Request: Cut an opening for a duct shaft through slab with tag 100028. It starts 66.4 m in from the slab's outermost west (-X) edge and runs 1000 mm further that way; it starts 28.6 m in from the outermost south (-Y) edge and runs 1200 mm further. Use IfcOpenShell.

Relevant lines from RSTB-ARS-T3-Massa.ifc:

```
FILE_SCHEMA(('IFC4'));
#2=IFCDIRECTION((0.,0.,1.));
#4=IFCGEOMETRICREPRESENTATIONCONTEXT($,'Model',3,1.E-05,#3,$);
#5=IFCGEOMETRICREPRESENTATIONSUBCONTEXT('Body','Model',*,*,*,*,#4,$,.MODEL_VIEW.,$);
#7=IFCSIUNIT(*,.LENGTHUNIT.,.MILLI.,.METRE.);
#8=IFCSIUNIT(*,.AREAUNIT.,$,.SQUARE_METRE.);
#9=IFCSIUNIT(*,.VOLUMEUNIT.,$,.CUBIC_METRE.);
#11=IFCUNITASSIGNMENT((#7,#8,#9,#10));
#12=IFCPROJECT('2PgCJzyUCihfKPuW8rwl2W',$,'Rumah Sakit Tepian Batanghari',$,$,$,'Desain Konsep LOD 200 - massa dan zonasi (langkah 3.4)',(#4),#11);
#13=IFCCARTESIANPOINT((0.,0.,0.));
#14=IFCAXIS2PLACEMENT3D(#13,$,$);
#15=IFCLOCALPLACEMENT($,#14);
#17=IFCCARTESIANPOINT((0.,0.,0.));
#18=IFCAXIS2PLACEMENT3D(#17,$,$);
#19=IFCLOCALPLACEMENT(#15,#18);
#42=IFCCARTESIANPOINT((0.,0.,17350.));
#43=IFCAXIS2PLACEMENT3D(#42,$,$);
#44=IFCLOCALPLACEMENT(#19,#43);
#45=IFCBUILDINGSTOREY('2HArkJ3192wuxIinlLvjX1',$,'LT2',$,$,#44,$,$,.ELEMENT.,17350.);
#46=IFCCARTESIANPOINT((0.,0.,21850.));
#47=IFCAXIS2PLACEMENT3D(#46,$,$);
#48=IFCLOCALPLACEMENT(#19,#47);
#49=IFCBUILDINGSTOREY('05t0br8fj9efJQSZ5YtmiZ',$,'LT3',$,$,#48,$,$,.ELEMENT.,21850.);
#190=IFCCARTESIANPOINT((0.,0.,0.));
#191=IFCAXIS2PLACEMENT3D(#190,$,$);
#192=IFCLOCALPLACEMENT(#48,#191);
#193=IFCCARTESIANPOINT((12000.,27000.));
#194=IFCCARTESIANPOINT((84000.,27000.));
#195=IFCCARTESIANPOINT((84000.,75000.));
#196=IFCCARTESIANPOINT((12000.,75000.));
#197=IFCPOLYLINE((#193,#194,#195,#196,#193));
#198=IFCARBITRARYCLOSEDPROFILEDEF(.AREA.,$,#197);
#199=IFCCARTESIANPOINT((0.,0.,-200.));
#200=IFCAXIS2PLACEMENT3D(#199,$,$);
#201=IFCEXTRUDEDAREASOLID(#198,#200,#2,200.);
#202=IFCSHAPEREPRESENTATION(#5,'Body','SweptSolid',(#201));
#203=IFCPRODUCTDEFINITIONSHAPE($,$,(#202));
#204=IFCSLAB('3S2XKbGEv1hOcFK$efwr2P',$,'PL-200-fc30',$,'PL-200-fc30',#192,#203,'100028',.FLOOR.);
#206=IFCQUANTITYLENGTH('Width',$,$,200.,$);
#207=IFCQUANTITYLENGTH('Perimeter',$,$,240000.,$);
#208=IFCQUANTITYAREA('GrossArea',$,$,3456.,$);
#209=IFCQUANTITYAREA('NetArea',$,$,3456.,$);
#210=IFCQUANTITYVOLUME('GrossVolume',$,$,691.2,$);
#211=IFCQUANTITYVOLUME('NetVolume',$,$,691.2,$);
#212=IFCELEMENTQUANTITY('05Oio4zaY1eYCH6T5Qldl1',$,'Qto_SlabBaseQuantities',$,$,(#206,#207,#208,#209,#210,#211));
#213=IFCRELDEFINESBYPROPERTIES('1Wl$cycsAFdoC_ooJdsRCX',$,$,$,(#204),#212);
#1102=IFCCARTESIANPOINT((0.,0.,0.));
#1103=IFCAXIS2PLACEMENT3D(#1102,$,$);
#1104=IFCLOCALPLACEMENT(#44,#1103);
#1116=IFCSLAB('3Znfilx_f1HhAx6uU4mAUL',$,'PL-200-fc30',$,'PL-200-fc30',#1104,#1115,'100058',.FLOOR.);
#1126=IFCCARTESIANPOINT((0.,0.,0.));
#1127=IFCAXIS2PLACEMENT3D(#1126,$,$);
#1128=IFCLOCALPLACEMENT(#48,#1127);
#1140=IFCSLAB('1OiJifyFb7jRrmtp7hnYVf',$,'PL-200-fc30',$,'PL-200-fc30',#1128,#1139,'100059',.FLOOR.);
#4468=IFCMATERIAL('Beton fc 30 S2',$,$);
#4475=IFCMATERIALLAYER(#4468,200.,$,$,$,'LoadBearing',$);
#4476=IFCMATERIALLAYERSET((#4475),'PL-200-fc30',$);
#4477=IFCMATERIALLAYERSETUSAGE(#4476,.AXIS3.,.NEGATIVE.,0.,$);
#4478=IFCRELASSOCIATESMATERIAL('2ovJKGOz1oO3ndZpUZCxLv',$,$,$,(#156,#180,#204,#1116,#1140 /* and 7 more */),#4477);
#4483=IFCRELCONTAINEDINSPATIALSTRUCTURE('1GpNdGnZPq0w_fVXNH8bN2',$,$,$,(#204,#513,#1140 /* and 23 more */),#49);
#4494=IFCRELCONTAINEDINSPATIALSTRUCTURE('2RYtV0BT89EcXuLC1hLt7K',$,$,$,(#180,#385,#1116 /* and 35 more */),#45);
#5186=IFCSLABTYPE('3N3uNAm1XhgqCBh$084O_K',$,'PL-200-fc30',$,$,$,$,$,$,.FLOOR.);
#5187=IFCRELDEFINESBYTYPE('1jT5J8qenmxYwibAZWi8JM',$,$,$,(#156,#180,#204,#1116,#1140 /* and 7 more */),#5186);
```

```python
import numpy as np
import ifcopenshell
import ifcopenshell.api.feature
import ifcopenshell.api.geometry
import ifcopenshell.api.pset
import ifcopenshell.api.root
import ifcopenshell.geom
import ifcopenshell.util.element
import ifcopenshell.util.placement
import ifcopenshell.util.representation
import ifcopenshell.util.shape
import ifcopenshell.util.unit

model = ifcopenshell.open("RSTB-ARS-T3-Massa.ifc")
unit_scale = ifcopenshell.util.unit.calculate_unit_scale(model)
area_scale = ifcopenshell.util.unit.calculate_unit_scale(model, "AREAUNIT")
volume_scale = ifcopenshell.util.unit.calculate_unit_scale(model, "VOLUMEUNIT")
settings = ifcopenshell.geom.settings()


def volume(element):
    """Net volume in cubic metres, openings subtracted."""
    shape = ifcopenshell.geom.create_shape(settings, element)
    return ifcopenshell.util.shape.get_volume(shape.geometry)


slab = model.by_guid("3S2XKbGEv1hOcFK$efwr2P")
before = volume(slab)

# Extent in the slab's own axes, in metres. The edges named are its -X and -Y sides.
slab_shape = ifcopenshell.geom.create_shape(settings, slab)
vertices = ifcopenshell.util.shape.get_vertices(slab_shape.geometry)
x_min, y_min, bottom = vertices.min(axis=0)
top = vertices[:, 2].max()

opening = ifcopenshell.api.root.create_entity(model, ifc_class="IfcOpeningElement", name="Duct shaft opening", predefined_type="OPENING")
context = ifcopenshell.util.representation.get_context(model, "Model", "Body", "MODEL_VIEW")
width, depth = 1, 1.2
outline = [(0.0, 0.0), (width, 0.0), (width, depth), (0.0, depth), (0.0, 0.0)]
# Overshoot both faces by 50 mm so the cut is clean.
shape = ifcopenshell.api.geometry.add_slab_representation(
    model, context=context, depth=top - bottom + 0.1, polyline=outline
)
ifcopenshell.api.geometry.assign_representation(model, product=opening, representation=shape)

matrix = ifcopenshell.util.placement.get_local_placement(slab.ObjectPlacement)
matrix[:, 3] = matrix @ np.append(np.array([x_min + 66.4, y_min + 28.6, bottom - 0.05]) / unit_scale, 1.0)
ifcopenshell.api.geometry.edit_object_placement(model, product=opening, matrix=matrix, is_si=False)
ifcopenshell.api.feature.add_feature(model, feature=opening, element=slab)

after = volume(slab)

# Update the slab's stored quantities.
qto = model.by_id(ifcopenshell.util.element.get_pset(slab, "Qto_SlabBaseQuantities", should_inherit=False)["id"])
ifcopenshell.api.pset.edit_qto(model, qto=qto, properties={
    "NetArea": after / (top - bottom) / area_scale,
    "NetVolume": after / volume_scale,
})

print(f"slab volume {before:.3f} -> {after:.3f} m3")

model.write("RSTB-ARS-T3-Massa_edited.ifc")
```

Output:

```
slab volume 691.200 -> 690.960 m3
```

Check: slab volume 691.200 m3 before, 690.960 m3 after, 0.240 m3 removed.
